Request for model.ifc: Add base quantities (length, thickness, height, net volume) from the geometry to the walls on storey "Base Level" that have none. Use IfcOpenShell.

First a look at what the model holds.

```python
import ifcopenshell
import ifcopenshell.util.element
import ifcopenshell.util.unit

model = ifcopenshell.open("model.ifc")
print(model.schema)
for unit_type in ("LENGTHUNIT", "AREAUNIT", "VOLUMEUNIT"):
    print(unit_type, ifcopenshell.util.unit.calculate_unit_scale(model, unit_type))
storey = next(s for s in model.by_type("IfcBuildingStorey") if s.Name == "Base Level")
walls = [e for e in ifcopenshell.util.element.get_decomposition(storey) if e.is_a("IfcWall")]
for e in sorted(walls, key=lambda e: e.id()):
    print(e.id(), e.is_a(), e.Name, list(ifcopenshell.util.element.get_psets(e, qtos_only=True)), sep=" | ")
```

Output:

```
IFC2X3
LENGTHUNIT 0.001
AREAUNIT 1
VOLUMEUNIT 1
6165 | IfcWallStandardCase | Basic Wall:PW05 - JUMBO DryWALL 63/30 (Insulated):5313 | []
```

```python
import ifcopenshell
import ifcopenshell.api.pset
import ifcopenshell.geom
import ifcopenshell.util.element
import ifcopenshell.util.shape
import ifcopenshell.util.unit

model = ifcopenshell.open("model.ifc")
unit_scale = ifcopenshell.util.unit.calculate_unit_scale(model)
volume_scale = ifcopenshell.util.unit.calculate_unit_scale(model, "VOLUMEUNIT")
settings = ifcopenshell.geom.settings()

storey = next(s for s in model.by_type("IfcBuildingStorey") if s.Name == "Base Level")
walls = [e for e in ifcopenshell.util.element.get_decomposition(storey) if e.is_a("IfcWall")]

for e in sorted(walls, key=lambda e: e.id()):
    if ifcopenshell.util.element.get_psets(e, qtos_only=True, should_inherit=False):
        continue
    # Geometry comes back in metres, in the element's own axes.
    shape = ifcopenshell.geom.create_shape(settings, e)
    values = {
        "Length": ifcopenshell.util.shape.get_x(shape.geometry) / unit_scale,
        "Width": ifcopenshell.util.shape.get_y(shape.geometry) / unit_scale,
        "Height": ifcopenshell.util.shape.get_z(shape.geometry) / unit_scale,
        "NetVolume": ifcopenshell.util.shape.get_volume(shape.geometry) / volume_scale,
    }
    qto = ifcopenshell.api.pset.add_qto(model, product=e, name="BaseQuantities")
    ifcopenshell.api.pset.edit_qto(model, qto=qto, properties=values)
    print(e.id(), {k: round(v, 3) for k, v in values.items()})

model.write("model_updated.ifc")
```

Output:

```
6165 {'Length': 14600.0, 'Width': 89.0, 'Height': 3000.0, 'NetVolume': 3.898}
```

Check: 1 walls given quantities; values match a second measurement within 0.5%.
